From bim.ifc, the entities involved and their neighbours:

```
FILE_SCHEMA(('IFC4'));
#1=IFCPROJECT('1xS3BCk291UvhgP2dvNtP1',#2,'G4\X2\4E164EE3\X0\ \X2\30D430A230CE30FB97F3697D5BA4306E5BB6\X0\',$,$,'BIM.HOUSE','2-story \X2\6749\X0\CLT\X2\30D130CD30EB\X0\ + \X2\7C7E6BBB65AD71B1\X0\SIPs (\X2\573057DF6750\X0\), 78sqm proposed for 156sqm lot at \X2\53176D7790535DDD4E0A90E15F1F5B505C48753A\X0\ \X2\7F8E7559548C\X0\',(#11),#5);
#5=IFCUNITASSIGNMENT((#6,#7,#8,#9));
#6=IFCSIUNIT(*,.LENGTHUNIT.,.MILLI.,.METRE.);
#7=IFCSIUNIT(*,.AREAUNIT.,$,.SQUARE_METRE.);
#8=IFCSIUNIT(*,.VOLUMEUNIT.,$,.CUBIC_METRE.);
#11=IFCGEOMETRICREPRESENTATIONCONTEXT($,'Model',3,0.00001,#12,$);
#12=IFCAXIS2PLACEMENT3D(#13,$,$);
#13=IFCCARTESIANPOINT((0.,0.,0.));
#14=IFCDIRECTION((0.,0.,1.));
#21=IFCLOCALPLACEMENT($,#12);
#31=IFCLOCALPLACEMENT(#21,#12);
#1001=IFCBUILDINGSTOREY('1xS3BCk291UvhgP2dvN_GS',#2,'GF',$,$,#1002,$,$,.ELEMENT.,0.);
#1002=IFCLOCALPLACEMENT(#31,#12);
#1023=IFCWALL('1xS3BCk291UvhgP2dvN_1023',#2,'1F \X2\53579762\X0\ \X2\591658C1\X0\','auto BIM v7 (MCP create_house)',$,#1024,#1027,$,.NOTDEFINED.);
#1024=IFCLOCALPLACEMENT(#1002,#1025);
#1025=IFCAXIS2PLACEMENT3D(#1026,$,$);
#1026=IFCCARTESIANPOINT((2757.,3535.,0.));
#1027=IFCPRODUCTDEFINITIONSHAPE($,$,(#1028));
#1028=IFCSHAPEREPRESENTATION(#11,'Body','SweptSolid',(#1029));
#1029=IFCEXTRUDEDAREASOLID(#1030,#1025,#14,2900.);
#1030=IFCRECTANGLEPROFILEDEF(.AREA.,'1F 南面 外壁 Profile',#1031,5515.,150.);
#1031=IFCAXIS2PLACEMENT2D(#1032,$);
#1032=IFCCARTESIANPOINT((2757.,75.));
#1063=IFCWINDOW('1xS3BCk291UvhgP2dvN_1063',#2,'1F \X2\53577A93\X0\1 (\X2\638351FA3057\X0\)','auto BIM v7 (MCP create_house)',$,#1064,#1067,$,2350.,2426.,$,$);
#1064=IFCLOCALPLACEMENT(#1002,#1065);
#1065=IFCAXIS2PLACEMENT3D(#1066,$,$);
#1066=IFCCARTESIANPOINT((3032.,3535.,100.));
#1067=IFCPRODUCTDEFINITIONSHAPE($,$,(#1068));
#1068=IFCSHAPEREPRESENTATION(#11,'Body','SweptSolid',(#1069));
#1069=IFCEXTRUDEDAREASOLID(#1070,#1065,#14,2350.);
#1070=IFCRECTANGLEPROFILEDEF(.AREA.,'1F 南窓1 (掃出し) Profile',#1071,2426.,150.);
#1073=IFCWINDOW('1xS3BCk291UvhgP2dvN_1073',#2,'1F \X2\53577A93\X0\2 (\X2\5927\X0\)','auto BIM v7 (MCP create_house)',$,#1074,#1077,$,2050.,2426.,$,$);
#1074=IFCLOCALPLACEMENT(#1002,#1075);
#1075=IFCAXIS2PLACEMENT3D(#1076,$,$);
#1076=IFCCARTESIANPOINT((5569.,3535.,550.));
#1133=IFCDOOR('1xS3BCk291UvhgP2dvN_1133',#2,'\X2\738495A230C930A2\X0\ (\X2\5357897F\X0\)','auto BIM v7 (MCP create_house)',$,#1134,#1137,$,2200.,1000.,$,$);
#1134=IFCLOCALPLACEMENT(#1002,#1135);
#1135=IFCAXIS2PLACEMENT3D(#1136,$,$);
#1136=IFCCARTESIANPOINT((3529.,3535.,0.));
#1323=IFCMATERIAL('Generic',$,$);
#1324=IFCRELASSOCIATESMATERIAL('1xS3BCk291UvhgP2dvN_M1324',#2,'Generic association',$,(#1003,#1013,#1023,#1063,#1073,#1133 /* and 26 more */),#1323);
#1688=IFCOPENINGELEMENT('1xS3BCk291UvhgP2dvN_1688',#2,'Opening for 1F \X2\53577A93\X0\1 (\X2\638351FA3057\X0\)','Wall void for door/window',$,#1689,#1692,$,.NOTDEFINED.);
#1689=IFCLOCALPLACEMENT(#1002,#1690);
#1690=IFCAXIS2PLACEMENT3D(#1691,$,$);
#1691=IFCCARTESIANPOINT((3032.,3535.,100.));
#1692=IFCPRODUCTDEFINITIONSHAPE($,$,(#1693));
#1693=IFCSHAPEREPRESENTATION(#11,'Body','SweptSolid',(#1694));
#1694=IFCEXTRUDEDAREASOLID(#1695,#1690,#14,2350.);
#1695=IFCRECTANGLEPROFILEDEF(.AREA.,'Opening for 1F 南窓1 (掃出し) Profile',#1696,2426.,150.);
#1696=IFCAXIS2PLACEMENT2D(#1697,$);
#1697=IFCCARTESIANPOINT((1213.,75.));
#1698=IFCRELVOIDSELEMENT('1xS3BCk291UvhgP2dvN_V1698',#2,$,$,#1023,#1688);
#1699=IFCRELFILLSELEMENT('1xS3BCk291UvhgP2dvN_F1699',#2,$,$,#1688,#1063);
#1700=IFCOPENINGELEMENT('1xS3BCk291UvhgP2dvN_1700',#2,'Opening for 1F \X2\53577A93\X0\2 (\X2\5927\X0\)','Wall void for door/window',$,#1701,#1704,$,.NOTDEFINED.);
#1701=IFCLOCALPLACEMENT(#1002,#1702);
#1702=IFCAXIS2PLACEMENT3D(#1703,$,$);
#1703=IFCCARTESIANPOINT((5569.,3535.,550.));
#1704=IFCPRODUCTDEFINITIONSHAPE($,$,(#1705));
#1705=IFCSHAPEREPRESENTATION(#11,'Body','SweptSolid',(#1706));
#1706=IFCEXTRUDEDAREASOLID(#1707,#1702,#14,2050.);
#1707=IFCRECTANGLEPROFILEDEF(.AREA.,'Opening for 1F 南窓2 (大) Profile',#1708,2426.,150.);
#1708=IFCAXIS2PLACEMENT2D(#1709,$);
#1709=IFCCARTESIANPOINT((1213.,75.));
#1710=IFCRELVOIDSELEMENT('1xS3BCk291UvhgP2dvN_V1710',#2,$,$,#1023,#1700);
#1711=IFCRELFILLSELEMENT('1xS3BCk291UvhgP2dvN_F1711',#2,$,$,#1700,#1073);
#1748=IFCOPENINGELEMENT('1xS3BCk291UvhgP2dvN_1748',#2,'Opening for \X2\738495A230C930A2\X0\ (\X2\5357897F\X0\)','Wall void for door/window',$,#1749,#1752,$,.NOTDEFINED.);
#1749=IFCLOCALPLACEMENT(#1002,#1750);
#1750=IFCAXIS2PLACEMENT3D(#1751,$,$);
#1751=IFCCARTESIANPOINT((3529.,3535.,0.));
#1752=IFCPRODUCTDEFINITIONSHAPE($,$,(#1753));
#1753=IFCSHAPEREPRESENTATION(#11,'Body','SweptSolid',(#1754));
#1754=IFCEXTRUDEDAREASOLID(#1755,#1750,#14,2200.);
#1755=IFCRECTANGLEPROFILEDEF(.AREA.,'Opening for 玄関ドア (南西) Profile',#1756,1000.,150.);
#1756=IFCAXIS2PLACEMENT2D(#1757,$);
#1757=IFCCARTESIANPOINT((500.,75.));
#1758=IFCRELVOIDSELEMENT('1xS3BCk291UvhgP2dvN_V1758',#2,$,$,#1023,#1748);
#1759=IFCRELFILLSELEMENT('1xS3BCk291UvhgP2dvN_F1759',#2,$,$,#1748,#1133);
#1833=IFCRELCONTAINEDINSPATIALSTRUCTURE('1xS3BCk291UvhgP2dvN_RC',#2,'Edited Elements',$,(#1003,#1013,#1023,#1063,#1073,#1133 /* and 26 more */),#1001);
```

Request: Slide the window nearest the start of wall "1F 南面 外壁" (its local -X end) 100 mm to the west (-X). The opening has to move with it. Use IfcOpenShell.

```python
import ifcopenshell
import ifcopenshell.api.geometry
import ifcopenshell.util.placement
import ifcopenshell.util.unit

model = ifcopenshell.open("bim.ifc")
unit_scale = ifcopenshell.util.unit.calculate_unit_scale(model)

window = model.by_guid("1xS3BCk291UvhgP2dvN_1063")
opening = window.FillsVoids[0].RelatingOpeningElement
wall = opening.VoidsElements[0].RelatingBuildingElement

wall_matrix = ifcopenshell.util.placement.get_local_placement(wall.ObjectPlacement)
shift = wall_matrix[:3, 0] * -0.1 / unit_scale
before = ifcopenshell.util.placement.get_local_placement(window.ObjectPlacement)[:3, 3].copy()

# The window is not placed relative to its opening, so move both.
for product in (opening, window):
    matrix = ifcopenshell.util.placement.get_local_placement(product.ObjectPlacement)
    matrix[:3, 3] += shift
    ifcopenshell.api.geometry.edit_object_placement(model, product=product, matrix=matrix, is_si=False)

after = ifcopenshell.util.placement.get_local_placement(window.ObjectPlacement)[:3, 3]
print("window moved by", (after - before).round(3) + 0.0)

model.write("bim_edited.ifc")
```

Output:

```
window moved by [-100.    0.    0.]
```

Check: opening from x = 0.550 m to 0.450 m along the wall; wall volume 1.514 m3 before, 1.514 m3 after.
